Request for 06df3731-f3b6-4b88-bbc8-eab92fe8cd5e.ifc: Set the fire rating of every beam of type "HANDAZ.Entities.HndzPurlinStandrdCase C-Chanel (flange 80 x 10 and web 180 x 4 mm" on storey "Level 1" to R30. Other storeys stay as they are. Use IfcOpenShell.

First a look at what the model holds.

```python
import ifcopenshell
import ifcopenshell.util.element

model = ifcopenshell.open("06df3731-f3b6-4b88-bbc8-eab92fe8cd5e.ifc")
print(model.schema)
storey = next(s for s in model.by_type("IfcBuildingStorey") if s.Name == "Level 1")
beams = [e for e in ifcopenshell.util.element.get_decomposition(storey) if e.is_a("IfcBeam")]
seen = {}
for e in beams:
    element_type = ifcopenshell.util.element.get_type(e)
    key = (element_type.Name if element_type != e and element_type else None, ifcopenshell.util.element.get_pset(e, "Pset_BeamCommon", "FireRating"))
    seen[key] = seen.get(key, 0) + 1
for (name, value), count in sorted(seen.items(), key=str):
    print(count, "x", name, "|", value)
```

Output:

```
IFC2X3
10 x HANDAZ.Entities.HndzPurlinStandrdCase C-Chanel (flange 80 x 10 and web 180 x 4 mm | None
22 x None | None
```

```python
import ifcopenshell
import ifcopenshell.api.pset
import ifcopenshell.util.element

model = ifcopenshell.open("06df3731-f3b6-4b88-bbc8-eab92fe8cd5e.ifc")

storey = next(s for s in model.by_type("IfcBuildingStorey") if s.Name == "Level 1")
beams = [e for e in ifcopenshell.util.element.get_decomposition(storey) if e.is_a("IfcBeam")]

count = 0
for e in beams:
    element_type = ifcopenshell.util.element.get_type(e)
    if element_type in (None, e) or element_type.Name != "HANDAZ.Entities.HndzPurlinStandrdCase C-Chanel (flange 80 x 10 and web 180 x 4 mm":
        continue
    # add_pset returns the element's existing set when there is one.
    pset = ifcopenshell.api.pset.add_pset(model, product=e, name="Pset_BeamCommon")
    ifcopenshell.api.pset.edit_pset(model, pset=pset, properties={"FireRating": "R30"})
    count += 1

print(count, "beams updated")

model.write("06df3731-f3b6-4b88-bbc8-eab92fe8cd5e-out.ifc")
```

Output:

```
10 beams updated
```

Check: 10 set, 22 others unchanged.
